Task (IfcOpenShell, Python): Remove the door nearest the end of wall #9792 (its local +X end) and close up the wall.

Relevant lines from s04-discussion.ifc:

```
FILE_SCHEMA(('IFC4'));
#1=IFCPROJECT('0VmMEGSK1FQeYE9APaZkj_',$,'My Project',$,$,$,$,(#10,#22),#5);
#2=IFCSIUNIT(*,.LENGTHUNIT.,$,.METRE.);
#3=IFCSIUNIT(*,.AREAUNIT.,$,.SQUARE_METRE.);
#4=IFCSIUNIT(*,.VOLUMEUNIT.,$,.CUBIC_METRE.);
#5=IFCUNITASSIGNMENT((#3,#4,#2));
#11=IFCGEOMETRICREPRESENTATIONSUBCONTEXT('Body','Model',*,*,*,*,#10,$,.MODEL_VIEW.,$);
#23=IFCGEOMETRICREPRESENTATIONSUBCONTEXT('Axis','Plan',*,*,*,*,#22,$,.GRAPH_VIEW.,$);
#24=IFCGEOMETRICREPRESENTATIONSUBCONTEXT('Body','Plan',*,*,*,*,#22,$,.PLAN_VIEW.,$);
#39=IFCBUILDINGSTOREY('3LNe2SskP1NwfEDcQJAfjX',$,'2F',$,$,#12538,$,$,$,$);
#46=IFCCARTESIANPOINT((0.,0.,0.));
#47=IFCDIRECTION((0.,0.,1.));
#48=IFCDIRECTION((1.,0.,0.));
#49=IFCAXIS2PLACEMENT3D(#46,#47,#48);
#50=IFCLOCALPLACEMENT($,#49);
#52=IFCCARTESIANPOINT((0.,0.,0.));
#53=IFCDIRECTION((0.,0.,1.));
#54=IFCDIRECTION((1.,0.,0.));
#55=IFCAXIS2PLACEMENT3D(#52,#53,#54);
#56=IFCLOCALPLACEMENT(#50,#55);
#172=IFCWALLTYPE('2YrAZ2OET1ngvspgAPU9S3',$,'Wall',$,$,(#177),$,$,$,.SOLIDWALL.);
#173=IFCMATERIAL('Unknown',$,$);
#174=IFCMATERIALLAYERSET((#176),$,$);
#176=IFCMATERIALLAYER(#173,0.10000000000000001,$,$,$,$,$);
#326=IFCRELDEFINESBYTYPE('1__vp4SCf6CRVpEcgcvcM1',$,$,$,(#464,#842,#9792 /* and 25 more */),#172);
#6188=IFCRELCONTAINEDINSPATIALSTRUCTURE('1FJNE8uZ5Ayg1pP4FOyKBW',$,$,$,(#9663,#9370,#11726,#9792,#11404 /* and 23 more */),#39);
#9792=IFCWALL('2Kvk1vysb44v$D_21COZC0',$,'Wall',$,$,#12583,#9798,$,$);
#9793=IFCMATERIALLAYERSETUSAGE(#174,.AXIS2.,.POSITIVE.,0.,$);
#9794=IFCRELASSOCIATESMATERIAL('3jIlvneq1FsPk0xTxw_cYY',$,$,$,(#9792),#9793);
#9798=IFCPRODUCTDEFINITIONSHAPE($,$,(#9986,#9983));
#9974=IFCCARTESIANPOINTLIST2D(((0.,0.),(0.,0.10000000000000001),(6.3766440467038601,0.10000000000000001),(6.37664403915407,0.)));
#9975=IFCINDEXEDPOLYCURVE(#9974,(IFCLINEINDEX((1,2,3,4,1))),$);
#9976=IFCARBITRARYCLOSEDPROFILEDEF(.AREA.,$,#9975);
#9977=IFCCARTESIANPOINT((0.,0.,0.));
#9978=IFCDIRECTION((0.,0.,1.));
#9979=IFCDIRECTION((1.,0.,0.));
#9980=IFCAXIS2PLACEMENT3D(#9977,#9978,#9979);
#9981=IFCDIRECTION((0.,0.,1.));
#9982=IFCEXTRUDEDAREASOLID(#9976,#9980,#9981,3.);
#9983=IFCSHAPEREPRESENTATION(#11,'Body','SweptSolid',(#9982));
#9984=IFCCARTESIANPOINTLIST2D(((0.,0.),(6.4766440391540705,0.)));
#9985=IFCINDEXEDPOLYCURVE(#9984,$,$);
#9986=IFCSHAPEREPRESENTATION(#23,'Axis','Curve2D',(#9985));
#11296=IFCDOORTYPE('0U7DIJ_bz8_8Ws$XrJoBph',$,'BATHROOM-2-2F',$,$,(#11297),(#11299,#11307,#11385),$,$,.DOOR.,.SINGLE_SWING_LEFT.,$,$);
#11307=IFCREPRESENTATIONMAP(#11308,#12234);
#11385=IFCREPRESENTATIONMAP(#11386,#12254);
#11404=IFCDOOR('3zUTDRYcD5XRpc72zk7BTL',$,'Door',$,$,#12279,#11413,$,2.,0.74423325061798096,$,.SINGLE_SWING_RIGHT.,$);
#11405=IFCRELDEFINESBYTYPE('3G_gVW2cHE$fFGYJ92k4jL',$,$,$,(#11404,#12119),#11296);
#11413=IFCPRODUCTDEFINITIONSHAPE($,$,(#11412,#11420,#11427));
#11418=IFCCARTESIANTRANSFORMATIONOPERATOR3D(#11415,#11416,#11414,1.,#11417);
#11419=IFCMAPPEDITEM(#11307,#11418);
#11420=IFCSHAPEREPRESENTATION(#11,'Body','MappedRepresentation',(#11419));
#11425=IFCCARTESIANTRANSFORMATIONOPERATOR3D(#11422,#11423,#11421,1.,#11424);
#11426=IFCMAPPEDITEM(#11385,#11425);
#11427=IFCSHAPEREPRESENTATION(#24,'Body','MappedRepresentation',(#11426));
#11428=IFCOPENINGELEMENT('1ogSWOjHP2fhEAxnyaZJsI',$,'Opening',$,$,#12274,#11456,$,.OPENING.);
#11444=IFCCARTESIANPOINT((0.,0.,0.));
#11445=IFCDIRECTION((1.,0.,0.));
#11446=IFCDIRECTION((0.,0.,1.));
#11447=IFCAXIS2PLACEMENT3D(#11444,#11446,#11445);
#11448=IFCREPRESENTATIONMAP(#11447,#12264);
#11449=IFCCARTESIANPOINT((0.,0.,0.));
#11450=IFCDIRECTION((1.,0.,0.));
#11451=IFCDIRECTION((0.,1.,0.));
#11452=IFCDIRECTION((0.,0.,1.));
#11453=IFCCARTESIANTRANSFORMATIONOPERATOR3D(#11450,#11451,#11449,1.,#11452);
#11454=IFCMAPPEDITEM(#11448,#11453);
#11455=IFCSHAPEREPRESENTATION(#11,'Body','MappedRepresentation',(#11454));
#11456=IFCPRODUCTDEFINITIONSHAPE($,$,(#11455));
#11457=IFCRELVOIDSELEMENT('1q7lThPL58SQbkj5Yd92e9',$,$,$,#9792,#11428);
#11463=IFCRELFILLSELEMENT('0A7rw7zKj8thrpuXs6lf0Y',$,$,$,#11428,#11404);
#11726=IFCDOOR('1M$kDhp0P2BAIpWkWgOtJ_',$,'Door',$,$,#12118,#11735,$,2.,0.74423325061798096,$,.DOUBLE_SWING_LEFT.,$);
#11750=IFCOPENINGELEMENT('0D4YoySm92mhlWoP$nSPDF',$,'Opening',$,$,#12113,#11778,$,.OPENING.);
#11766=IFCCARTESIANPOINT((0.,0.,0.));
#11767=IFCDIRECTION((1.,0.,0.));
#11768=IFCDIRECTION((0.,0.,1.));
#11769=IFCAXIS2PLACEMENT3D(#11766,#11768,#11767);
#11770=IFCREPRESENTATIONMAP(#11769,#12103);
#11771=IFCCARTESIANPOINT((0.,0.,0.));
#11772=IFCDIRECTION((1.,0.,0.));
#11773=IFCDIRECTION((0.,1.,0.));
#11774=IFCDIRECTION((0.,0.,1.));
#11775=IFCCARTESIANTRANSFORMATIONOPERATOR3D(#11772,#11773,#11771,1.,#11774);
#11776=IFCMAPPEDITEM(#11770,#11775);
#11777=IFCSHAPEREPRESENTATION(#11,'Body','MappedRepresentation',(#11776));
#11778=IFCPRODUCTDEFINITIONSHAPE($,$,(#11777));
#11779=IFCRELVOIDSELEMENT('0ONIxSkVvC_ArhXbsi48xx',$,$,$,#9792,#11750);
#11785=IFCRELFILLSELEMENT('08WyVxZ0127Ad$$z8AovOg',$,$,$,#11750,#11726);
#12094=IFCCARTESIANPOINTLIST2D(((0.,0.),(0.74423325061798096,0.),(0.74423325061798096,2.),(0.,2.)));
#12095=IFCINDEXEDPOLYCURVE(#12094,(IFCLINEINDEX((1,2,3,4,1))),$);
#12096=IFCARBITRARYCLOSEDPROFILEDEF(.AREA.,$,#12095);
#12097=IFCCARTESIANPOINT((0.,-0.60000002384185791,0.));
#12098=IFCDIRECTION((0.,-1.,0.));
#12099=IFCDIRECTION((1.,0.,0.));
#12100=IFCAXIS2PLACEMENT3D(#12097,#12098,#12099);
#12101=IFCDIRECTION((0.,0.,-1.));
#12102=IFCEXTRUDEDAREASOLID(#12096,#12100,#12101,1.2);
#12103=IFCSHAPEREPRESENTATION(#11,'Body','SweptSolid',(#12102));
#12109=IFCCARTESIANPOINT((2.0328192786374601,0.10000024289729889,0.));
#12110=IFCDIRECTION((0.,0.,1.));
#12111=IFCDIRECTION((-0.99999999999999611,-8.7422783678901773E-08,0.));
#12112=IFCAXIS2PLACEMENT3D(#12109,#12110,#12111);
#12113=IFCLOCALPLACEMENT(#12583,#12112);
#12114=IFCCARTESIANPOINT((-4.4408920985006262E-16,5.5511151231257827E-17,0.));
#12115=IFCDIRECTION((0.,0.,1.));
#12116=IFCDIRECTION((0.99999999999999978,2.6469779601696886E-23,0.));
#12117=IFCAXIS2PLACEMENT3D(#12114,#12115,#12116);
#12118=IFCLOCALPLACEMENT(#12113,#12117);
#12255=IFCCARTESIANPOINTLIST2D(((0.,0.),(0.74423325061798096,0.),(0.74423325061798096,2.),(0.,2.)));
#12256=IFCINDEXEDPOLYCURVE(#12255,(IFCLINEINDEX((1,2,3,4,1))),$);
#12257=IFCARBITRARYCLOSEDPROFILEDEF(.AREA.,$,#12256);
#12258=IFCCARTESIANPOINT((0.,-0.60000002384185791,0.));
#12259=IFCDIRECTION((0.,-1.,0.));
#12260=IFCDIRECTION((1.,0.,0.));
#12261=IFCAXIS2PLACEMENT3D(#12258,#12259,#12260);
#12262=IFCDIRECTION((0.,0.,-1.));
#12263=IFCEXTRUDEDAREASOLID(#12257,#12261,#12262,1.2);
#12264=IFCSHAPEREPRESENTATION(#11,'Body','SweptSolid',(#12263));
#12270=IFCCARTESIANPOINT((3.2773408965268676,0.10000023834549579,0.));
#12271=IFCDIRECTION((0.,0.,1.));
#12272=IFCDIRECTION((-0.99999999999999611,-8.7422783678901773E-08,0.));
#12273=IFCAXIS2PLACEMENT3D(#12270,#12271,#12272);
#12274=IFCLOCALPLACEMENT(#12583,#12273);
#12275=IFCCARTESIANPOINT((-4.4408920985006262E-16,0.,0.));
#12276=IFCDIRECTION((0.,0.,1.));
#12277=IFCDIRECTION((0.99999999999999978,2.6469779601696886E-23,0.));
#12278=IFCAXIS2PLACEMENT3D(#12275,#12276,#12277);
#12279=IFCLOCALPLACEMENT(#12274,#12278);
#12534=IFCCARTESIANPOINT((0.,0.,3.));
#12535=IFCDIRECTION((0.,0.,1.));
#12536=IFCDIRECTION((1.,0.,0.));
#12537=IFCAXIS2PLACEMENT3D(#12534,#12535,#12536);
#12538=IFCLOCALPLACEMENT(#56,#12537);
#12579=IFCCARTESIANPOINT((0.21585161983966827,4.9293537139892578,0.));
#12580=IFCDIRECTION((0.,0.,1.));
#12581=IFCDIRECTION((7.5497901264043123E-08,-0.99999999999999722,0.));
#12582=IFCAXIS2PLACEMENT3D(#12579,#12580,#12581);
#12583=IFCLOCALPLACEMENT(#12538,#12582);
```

```python
import ifcopenshell
import ifcopenshell.api.feature
import ifcopenshell.api.root
import ifcopenshell.geom
import ifcopenshell.util.shape

model = ifcopenshell.open("s04-discussion.ifc")
settings = ifcopenshell.geom.settings()


def volume(element):
    """Net volume in cubic metres, openings subtracted."""
    shape = ifcopenshell.geom.create_shape(settings, element)
    return ifcopenshell.util.shape.get_volume(shape.geometry)


door = model.by_guid("3zUTDRYcD5XRpc72zk7BTL")
opening = door.FillsVoids[0].RelatingOpeningElement
wall = opening.VoidsElements[0].RelatingBuildingElement
before = volume(wall)

ifcopenshell.api.root.remove_product(model, product=door)
ifcopenshell.api.feature.remove_feature(model, feature=opening)

after = volume(wall)

print(f"wall volume {before:.3f} -> {after:.3f} m3")

model.write("s04-discussion_updated.ifc")
```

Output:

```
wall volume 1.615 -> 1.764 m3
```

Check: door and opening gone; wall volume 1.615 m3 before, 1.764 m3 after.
